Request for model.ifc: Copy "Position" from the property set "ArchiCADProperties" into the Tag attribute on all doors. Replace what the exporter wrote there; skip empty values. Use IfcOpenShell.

First a look at what the model holds.

```python
import ifcopenshell
import ifcopenshell.util.element

model = ifcopenshell.open("model.ifc")
print(model.schema)
doors = model.by_type("IfcDoor")
print(len(doors), "doors")
for e in doors[:8]:
    source = ifcopenshell.util.element.get_pset(e, "ArchiCADProperties", "Position")
    target = e.Tag
    print(e.id(), repr(source), repr(target), sep=" | ")
```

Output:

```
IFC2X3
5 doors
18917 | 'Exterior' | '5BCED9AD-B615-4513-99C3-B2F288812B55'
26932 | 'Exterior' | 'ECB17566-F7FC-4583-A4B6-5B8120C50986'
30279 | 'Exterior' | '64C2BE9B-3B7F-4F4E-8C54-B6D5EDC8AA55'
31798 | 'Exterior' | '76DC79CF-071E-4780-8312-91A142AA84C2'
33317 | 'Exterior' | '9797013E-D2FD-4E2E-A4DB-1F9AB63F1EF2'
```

```python
import ifcopenshell
import ifcopenshell.util.element

model = ifcopenshell.open("model.ifc")

count = 0
for e in model.by_type("IfcDoor"):
    value = ifcopenshell.util.element.get_pset(e, "ArchiCADProperties", "Position")
    current = e.Tag
    if not value or not value.strip() or current == value:
        continue
    e.Tag = value
    count += 1

print(count, "doors updated")

model.write("model-out.ifc")
```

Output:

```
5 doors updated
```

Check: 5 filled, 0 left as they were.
